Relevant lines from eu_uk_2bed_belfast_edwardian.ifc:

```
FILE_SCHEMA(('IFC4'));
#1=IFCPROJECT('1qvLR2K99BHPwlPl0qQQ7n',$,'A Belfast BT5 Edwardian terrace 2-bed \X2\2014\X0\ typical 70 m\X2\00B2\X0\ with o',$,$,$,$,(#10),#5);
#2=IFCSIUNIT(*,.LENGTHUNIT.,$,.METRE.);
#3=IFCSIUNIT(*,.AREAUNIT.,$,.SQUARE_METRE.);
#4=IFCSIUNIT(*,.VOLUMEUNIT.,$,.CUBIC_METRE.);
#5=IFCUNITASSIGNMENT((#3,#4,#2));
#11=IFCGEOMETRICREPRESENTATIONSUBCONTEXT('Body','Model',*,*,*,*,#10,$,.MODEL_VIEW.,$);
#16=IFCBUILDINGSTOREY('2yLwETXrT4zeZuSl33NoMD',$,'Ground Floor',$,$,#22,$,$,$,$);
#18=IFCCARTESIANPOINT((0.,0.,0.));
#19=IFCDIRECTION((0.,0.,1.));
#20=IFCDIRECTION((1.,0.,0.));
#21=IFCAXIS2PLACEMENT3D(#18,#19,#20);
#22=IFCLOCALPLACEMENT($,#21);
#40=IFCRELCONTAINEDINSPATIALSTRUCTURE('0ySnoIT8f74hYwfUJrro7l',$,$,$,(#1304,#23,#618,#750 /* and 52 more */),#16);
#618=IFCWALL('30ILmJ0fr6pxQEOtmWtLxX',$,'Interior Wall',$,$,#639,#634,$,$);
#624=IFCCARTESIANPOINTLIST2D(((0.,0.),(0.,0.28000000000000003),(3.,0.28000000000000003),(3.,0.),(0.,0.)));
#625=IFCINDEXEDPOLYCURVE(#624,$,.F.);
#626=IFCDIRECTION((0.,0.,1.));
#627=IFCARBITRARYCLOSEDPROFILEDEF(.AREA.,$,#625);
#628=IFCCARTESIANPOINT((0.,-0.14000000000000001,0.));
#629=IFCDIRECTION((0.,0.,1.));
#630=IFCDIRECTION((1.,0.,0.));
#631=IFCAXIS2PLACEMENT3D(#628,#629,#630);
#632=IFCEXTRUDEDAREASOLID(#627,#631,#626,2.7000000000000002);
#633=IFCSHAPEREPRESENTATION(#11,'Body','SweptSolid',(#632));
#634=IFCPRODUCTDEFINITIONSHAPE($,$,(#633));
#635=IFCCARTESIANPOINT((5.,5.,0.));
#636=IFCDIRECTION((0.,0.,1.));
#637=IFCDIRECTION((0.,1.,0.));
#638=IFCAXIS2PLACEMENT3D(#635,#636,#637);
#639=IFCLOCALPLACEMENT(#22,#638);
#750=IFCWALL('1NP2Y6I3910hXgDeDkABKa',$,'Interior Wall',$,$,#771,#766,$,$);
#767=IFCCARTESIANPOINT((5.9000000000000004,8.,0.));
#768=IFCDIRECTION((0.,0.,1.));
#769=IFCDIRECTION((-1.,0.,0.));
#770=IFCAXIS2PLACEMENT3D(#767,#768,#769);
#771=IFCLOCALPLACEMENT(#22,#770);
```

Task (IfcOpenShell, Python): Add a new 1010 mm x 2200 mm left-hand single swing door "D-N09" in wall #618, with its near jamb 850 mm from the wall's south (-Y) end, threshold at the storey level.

```python
import numpy as np
import ifcopenshell
import ifcopenshell.api.feature
import ifcopenshell.api.geometry
import ifcopenshell.api.root
import ifcopenshell.api.spatial
import ifcopenshell.geom
import ifcopenshell.util.element
import ifcopenshell.util.placement
import ifcopenshell.util.representation
import ifcopenshell.util.shape
import ifcopenshell.util.unit

model = ifcopenshell.open("eu_uk_2bed_belfast_edwardian.ifc")
unit_scale = ifcopenshell.util.unit.calculate_unit_scale(model)
settings = ifcopenshell.geom.settings()


def volume(element):
    """Net volume in cubic metres, openings subtracted."""
    shape = ifcopenshell.geom.create_shape(settings, element)
    return ifcopenshell.util.shape.get_volume(shape.geometry)


wall = model.by_guid("30ILmJ0fr6pxQEOtmWtLxX")
storey = ifcopenshell.util.element.get_container(wall, ifc_class="IfcBuildingStorey")
context = ifcopenshell.util.representation.get_context(model, "Model", "Body", "MODEL_VIEW")
before = volume(wall)

width, height, from_end, sill = 1.01, 2.2, 0.85, 0.0  # metres

# The wall runs along its own X axis, and the end named is its -X end.
wall_shape = ifcopenshell.geom.create_shape(settings, wall)
x, y, z = ifcopenshell.util.shape.get_vertices(wall_shape.geometry).T
start = x.min() + from_end
face, thickness = float(y.min()), float(y.max() - y.min())
wall_matrix = ifcopenshell.util.placement.get_local_placement(wall.ObjectPlacement)
level = ifcopenshell.util.placement.get_local_placement(storey.ObjectPlacement)[2, 3]


def in_wall(x, y):
    """Placement at x, y metres in the wall's axes, at sill height."""
    matrix = wall_matrix.copy()
    matrix[:, 3] = wall_matrix @ np.array([x / unit_scale, y / unit_scale, 0.0, 1.0])
    matrix[2, 3] = level + sill / unit_scale
    return matrix


# Opening: a box that overshoots both wall faces by 50 mm.
opening = ifcopenshell.api.root.create_entity(model, ifc_class="IfcOpeningElement", predefined_type="OPENING")
box = ifcopenshell.api.geometry.add_wall_representation(
    model, context=context, length=width, height=height, thickness=thickness + 0.1
)
ifcopenshell.api.geometry.assign_representation(model, product=opening, representation=box)
ifcopenshell.api.geometry.edit_object_placement(model, product=opening, matrix=in_wall(start, face - 0.05), is_si=False)
ifcopenshell.api.feature.add_feature(model, feature=opening, element=wall)

door = ifcopenshell.api.root.create_entity(model, ifc_class="IfcDoor", name="D-N09", predefined_type="DOOR")
door.OverallWidth, door.OverallHeight = width / unit_scale, height / unit_scale
door.OperationType = "SINGLE_SWING_LEFT"
body = ifcopenshell.api.geometry.add_door_representation(
    model,
    context=context,
    overall_width=door.OverallWidth,
    overall_height=door.OverallHeight,
    operation_type="SINGLE_SWING_LEFT",
    lining_properties={"LiningDepth": thickness / unit_scale, "ThresholdDepth": thickness / unit_scale},
)
ifcopenshell.api.geometry.assign_representation(model, product=door, representation=body)
ifcopenshell.api.spatial.assign_container(model, products=[door], relating_structure=storey)
ifcopenshell.api.feature.add_filling(model, opening=opening, element=door)

# The lining spans the wall, so the door starts at the wall face.
ifcopenshell.api.geometry.edit_object_placement(model, product=door, matrix=in_wall(start, face), is_si=False)

after = volume(wall)

print(f"wall volume {before:.3f} -> {after:.3f} m3")

model.write("eu_uk_2bed_belfast_edwardian-out.ifc")
```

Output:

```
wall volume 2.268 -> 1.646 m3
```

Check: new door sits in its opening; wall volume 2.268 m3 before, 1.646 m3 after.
